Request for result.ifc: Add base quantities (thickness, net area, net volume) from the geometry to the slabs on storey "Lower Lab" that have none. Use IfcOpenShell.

First a look at what the model holds.

```python
import ifcopenshell
import ifcopenshell.util.element
import ifcopenshell.util.unit

model = ifcopenshell.open("result.ifc")
print(model.schema)
for unit_type in ("LENGTHUNIT", "AREAUNIT", "VOLUMEUNIT"):
    print(unit_type, ifcopenshell.util.unit.calculate_unit_scale(model, unit_type))
storey = next(s for s in model.by_type("IfcBuildingStorey") if s.Name == "Lower Lab")
slabs = [e for e in ifcopenshell.util.element.get_decomposition(storey) if e.is_a("IfcSlab")]
for e in sorted(slabs, key=lambda e: e.id()):
    print(e.id(), e.is_a(), e.Name, list(ifcopenshell.util.element.get_psets(e, qtos_only=True)), sep=" | ")
```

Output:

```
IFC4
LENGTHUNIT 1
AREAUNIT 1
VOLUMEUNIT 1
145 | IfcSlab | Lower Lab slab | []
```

```python
import ifcopenshell
import ifcopenshell.api.pset
import ifcopenshell.geom
import ifcopenshell.util.element
import ifcopenshell.util.shape
import ifcopenshell.util.unit

model = ifcopenshell.open("result.ifc")
unit_scale = ifcopenshell.util.unit.calculate_unit_scale(model)
area_scale = ifcopenshell.util.unit.calculate_unit_scale(model, "AREAUNIT")
volume_scale = ifcopenshell.util.unit.calculate_unit_scale(model, "VOLUMEUNIT")
settings = ifcopenshell.geom.settings()

storey = next(s for s in model.by_type("IfcBuildingStorey") if s.Name == "Lower Lab")
slabs = [e for e in ifcopenshell.util.element.get_decomposition(storey) if e.is_a("IfcSlab")]

for e in sorted(slabs, key=lambda e: e.id()):
    if ifcopenshell.util.element.get_psets(e, qtos_only=True, should_inherit=False):
        continue
    # Geometry comes back in metres, in the element's own axes.
    shape = ifcopenshell.geom.create_shape(settings, e)
    values = {
        "Width": ifcopenshell.util.shape.get_z(shape.geometry) / unit_scale,
        "NetArea": ifcopenshell.util.shape.get_footprint_area(shape.geometry) / area_scale,
        "NetVolume": ifcopenshell.util.shape.get_volume(shape.geometry) / volume_scale,
    }
    qto = ifcopenshell.api.pset.add_qto(model, product=e, name="Qto_SlabBaseQuantities")
    ifcopenshell.api.pset.edit_qto(model, qto=qto, properties=values)
    print(e.id(), {k: round(v, 3) for k, v in values.items()})

model.write("result_edited.ifc")
```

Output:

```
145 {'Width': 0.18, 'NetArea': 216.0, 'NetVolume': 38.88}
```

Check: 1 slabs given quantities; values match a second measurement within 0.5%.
